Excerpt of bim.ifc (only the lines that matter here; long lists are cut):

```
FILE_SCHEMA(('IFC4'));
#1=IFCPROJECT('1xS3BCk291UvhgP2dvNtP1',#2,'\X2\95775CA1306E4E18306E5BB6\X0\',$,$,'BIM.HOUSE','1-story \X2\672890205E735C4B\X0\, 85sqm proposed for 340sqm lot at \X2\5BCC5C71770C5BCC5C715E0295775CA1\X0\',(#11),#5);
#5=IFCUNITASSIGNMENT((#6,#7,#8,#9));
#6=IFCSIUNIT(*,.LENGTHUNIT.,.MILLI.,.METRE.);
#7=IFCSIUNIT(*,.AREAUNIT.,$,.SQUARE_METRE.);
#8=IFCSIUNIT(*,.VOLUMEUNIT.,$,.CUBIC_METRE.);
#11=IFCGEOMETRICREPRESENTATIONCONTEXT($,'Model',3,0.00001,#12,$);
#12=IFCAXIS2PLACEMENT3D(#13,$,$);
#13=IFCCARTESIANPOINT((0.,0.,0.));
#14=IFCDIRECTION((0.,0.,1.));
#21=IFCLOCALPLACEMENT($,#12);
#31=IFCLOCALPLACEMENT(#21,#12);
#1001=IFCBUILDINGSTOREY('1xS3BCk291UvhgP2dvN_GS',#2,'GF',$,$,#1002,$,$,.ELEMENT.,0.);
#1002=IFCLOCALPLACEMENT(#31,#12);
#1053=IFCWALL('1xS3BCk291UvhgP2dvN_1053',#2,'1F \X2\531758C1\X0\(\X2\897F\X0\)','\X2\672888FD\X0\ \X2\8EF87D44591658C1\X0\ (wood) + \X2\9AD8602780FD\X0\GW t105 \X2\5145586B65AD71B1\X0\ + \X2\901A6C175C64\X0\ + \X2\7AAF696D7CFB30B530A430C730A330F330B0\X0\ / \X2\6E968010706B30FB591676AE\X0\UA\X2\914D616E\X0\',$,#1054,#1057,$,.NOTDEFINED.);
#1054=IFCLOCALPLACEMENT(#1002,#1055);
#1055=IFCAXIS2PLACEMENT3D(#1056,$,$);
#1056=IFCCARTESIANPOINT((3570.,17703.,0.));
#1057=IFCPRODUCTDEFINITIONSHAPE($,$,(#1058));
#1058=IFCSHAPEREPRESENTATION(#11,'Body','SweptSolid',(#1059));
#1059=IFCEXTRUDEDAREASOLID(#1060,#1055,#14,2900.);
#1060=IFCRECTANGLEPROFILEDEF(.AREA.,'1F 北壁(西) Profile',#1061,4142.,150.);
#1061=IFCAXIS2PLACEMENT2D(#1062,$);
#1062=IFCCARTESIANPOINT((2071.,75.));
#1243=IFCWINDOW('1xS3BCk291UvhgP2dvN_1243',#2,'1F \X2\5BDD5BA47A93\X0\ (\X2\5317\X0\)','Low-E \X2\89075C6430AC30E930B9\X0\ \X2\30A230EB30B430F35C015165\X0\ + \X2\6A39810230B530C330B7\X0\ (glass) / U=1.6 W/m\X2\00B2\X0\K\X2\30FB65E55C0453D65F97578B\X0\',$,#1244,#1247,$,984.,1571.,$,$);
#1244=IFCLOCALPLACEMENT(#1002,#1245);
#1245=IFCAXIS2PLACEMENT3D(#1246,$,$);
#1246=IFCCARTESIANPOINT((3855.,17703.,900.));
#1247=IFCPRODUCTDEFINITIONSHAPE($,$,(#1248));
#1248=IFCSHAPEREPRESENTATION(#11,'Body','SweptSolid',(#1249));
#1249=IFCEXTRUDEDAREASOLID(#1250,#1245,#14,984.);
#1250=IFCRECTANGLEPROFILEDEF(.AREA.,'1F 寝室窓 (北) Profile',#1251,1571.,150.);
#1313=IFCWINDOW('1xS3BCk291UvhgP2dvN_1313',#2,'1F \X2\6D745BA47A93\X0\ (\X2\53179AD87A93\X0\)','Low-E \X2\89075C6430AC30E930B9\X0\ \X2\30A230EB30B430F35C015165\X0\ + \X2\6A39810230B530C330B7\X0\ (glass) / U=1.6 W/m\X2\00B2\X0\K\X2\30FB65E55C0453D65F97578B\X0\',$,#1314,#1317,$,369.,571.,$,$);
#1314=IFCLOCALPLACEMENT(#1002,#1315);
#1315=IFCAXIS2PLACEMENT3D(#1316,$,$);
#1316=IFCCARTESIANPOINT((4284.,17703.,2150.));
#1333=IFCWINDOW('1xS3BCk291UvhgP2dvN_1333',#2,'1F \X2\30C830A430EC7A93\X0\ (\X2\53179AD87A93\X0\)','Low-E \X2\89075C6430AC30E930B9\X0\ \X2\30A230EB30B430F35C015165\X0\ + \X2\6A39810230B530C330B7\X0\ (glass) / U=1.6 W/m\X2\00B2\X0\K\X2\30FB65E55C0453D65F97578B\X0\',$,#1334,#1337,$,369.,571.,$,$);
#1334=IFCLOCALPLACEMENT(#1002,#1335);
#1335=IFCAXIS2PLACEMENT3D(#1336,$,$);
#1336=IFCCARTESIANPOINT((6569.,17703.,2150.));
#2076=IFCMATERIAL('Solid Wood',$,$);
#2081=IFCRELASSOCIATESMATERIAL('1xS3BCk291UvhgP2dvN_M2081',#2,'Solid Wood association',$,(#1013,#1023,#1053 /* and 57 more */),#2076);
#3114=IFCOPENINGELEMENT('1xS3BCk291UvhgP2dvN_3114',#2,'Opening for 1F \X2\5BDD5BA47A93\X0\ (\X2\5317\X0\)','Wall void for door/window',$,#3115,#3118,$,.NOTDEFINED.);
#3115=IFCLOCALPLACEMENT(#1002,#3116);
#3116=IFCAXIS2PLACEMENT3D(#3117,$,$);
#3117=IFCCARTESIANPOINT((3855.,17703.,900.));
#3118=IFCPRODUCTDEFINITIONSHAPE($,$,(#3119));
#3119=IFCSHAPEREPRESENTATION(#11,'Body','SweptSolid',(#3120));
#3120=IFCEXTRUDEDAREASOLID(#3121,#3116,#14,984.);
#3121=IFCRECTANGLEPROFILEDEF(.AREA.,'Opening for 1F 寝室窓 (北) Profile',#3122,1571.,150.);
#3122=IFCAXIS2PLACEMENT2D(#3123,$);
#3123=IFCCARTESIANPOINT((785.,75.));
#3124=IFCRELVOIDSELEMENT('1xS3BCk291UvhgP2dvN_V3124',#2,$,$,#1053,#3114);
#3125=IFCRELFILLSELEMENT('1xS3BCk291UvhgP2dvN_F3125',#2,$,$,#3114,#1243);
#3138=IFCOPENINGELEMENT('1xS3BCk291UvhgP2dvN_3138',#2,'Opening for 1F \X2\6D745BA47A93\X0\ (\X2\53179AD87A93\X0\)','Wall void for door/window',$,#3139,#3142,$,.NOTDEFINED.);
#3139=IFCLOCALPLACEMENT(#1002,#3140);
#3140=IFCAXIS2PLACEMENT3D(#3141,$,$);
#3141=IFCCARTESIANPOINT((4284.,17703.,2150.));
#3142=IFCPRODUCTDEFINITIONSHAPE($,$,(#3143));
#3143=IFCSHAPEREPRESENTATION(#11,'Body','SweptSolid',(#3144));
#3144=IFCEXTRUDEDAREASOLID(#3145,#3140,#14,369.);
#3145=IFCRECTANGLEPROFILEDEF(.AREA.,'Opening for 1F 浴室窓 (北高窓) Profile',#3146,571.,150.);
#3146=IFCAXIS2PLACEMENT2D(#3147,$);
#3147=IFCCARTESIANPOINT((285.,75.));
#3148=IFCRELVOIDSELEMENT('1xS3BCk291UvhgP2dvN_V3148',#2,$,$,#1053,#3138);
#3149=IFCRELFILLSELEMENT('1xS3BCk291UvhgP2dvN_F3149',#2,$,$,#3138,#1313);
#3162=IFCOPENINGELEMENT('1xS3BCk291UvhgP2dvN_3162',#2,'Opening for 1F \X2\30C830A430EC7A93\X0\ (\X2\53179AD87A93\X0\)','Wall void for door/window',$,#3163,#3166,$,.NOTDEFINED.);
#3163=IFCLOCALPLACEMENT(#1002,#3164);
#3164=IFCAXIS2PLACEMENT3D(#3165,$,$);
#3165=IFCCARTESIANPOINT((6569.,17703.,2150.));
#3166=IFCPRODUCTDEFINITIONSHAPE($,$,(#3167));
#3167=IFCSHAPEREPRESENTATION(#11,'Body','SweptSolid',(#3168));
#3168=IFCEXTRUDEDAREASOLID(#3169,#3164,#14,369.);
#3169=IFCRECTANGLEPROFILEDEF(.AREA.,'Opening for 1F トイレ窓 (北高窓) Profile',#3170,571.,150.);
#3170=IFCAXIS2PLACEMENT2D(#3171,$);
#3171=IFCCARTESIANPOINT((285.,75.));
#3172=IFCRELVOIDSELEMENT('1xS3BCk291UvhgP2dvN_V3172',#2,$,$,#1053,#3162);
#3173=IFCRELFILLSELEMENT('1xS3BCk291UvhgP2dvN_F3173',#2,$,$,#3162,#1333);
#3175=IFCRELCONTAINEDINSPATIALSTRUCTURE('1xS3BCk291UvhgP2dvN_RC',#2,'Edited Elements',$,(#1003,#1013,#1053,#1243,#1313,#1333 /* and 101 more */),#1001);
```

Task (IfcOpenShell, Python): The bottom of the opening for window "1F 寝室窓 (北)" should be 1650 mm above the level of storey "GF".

```python
import numpy as np
import ifcopenshell
import ifcopenshell.api.geometry
import ifcopenshell.geom
import ifcopenshell.util.element
import ifcopenshell.util.placement
import ifcopenshell.util.shape
import ifcopenshell.util.unit

model = ifcopenshell.open("bim.ifc")
unit_scale = ifcopenshell.util.unit.calculate_unit_scale(model)

window = model.by_guid("1xS3BCk291UvhgP2dvN_1243")
opening = window.FillsVoids[0].RelatingOpeningElement
storey = ifcopenshell.util.element.get_container(window, ifc_class="IfcBuildingStorey")
level = ifcopenshell.util.placement.get_local_placement(storey.ObjectPlacement)[2, 3]

# The opening's origin need not be at the sill, so measure its lowest point.
shape = ifcopenshell.geom.create_shape(ifcopenshell.geom.settings(), opening)
bottom = ifcopenshell.util.shape.get_shape_bottom_elevation(shape, shape.geometry) / unit_scale
dz = level + 1650.0 - bottom

shift = np.array([0.0, 0.0, dz])
# The window is not placed relative to its opening, so move both.
for product in (opening, window):
    matrix = ifcopenshell.util.placement.get_local_placement(product.ObjectPlacement)
    matrix[:3, 3] += shift
    ifcopenshell.api.geometry.edit_object_placement(model, product=product, matrix=matrix, is_si=False)

print(f"moved by {dz * unit_scale:+.3f} m")

model.write("bim_rev.ifc")
```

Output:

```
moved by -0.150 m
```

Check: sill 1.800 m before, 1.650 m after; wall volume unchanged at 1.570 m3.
